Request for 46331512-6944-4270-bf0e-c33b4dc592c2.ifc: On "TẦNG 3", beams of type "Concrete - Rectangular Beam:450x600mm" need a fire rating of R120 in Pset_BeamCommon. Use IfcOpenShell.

First a look at what the model holds.

```python
import ifcopenshell
import ifcopenshell.util.element

model = ifcopenshell.open("46331512-6944-4270-bf0e-c33b4dc592c2.ifc")
print(model.schema)
storey = next(s for s in model.by_type("IfcBuildingStorey") if s.Name == "TẦNG 3")
beams = [e for e in ifcopenshell.util.element.get_decomposition(storey) if e.is_a("IfcBeam")]
seen = {}
for e in beams:
    element_type = ifcopenshell.util.element.get_type(e)
    key = (element_type.Name if element_type != e and element_type else None, ifcopenshell.util.element.get_pset(e, "Pset_BeamCommon", "FireRating"))
    seen[key] = seen.get(key, 0) + 1
for (name, value), count in sorted(seen.items(), key=str):
    print(count, "x", name, "|", value)
```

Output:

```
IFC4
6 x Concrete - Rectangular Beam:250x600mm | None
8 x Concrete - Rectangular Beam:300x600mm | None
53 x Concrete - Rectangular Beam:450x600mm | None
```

```python
import ifcopenshell
import ifcopenshell.api.pset
import ifcopenshell.util.element

model = ifcopenshell.open("46331512-6944-4270-bf0e-c33b4dc592c2.ifc")

storey = next(s for s in model.by_type("IfcBuildingStorey") if s.Name == "TẦNG 3")
beams = [e for e in ifcopenshell.util.element.get_decomposition(storey) if e.is_a("IfcBeam")]

count = 0
for e in beams:
    element_type = ifcopenshell.util.element.get_type(e)
    if element_type in (None, e) or element_type.Name != "Concrete - Rectangular Beam:450x600mm":
        continue
    # add_pset returns the element's existing set when there is one.
    pset = ifcopenshell.api.pset.add_pset(model, product=e, name="Pset_BeamCommon")
    ifcopenshell.api.pset.edit_pset(model, pset=pset, properties={"FireRating": "R120"})
    count += 1

print(count, "beams updated")

model.write("46331512-6944-4270-bf0e-c33b4dc592c2-out.ifc")
```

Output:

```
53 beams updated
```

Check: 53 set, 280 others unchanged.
